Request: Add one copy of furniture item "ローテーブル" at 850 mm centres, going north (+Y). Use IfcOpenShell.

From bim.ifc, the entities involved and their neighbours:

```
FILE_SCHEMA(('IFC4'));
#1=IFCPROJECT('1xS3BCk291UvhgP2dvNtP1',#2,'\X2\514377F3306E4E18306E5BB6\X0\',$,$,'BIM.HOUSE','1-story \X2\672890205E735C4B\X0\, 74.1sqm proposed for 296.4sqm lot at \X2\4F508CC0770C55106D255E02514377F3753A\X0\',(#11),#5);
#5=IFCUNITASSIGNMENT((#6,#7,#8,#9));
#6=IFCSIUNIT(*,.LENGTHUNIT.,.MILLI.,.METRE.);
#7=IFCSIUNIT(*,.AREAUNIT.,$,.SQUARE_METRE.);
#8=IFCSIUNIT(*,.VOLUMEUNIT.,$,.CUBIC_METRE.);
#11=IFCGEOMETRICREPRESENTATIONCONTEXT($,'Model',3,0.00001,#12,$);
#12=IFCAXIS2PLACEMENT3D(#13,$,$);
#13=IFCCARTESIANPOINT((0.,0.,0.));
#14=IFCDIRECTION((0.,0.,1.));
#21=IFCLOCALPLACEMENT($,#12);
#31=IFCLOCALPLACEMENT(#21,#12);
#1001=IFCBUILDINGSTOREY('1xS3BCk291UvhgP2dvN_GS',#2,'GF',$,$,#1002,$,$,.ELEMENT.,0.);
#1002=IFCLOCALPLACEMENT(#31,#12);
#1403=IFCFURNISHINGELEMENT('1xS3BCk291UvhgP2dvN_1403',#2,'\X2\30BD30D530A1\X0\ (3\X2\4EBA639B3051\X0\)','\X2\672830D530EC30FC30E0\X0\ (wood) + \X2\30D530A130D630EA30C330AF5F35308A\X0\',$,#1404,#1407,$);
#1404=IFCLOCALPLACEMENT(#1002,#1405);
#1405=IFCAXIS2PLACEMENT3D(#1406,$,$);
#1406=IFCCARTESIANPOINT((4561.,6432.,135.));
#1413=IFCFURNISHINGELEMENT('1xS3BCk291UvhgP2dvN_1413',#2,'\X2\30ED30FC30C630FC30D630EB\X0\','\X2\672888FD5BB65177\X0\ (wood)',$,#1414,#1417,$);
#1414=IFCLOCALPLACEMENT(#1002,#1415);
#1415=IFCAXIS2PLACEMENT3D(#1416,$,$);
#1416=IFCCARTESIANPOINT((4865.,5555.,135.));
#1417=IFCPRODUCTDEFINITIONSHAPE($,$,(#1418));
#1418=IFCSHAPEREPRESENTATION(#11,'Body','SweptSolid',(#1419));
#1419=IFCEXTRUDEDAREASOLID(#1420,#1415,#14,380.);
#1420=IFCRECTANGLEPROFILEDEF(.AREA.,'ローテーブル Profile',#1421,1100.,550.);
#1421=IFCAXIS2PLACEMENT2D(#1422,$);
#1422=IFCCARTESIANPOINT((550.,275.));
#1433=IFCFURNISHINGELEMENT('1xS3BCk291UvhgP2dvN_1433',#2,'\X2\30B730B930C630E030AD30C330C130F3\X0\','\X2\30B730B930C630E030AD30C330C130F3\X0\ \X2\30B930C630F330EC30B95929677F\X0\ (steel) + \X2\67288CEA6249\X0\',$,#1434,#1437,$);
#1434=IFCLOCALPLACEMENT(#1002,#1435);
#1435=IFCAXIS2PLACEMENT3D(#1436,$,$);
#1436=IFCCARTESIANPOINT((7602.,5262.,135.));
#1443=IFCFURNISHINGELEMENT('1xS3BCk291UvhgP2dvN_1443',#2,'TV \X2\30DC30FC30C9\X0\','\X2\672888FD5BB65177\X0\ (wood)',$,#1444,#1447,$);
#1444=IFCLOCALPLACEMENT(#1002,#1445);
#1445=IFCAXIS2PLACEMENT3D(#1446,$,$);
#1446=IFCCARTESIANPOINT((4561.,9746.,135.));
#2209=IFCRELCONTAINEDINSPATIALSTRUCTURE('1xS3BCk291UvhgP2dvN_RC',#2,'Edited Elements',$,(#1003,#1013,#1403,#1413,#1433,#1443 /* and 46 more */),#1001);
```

```python
import numpy as np
import ifcopenshell
import ifcopenshell.api.geometry
import ifcopenshell.api.root
import ifcopenshell.util.element
import ifcopenshell.util.placement
import ifcopenshell.util.unit

model = ifcopenshell.open("bim.ifc")
unit_scale = ifcopenshell.util.unit.calculate_unit_scale(model)


def reuse_history(source, copy):
    """copy_class also copies each property set's owner history, people and application; keep the originals."""
    for rel in copy.IsDefinedBy:
        if rel.is_a("IfcRelDefinesByProperties") and (history := rel.RelatingPropertyDefinition.OwnerHistory):
            rel.RelatingPropertyDefinition.OwnerHistory = source.OwnerHistory
            ifcopenshell.util.element.remove_deep2(model, history)


source = model.by_guid("1xS3BCk291UvhgP2dvN_1413")
base = ifcopenshell.util.placement.get_local_placement(source.ObjectPlacement)
step = np.array([0.0, 1.0, 0.0]) * 0.85 / unit_scale

for i in range(1, 2):
    copy = ifcopenshell.api.root.copy_class(model, product=source)
    copy.Representation = ifcopenshell.util.element.copy_deep(
        model, source.Representation, exclude=["IfcGeometricRepresentationContext", "IfcRepresentationMap"]
    )
    reuse_history(source, copy)
    matrix = base.copy()
    matrix[:3, 3] += i * step
    print("added at", matrix[:3, 3].round(3) + 0.0)
    ifcopenshell.api.geometry.edit_object_placement(model, product=copy, matrix=matrix, is_si=False)

model.write("bim_edited.ifc")
```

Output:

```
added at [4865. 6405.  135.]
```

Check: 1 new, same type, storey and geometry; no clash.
